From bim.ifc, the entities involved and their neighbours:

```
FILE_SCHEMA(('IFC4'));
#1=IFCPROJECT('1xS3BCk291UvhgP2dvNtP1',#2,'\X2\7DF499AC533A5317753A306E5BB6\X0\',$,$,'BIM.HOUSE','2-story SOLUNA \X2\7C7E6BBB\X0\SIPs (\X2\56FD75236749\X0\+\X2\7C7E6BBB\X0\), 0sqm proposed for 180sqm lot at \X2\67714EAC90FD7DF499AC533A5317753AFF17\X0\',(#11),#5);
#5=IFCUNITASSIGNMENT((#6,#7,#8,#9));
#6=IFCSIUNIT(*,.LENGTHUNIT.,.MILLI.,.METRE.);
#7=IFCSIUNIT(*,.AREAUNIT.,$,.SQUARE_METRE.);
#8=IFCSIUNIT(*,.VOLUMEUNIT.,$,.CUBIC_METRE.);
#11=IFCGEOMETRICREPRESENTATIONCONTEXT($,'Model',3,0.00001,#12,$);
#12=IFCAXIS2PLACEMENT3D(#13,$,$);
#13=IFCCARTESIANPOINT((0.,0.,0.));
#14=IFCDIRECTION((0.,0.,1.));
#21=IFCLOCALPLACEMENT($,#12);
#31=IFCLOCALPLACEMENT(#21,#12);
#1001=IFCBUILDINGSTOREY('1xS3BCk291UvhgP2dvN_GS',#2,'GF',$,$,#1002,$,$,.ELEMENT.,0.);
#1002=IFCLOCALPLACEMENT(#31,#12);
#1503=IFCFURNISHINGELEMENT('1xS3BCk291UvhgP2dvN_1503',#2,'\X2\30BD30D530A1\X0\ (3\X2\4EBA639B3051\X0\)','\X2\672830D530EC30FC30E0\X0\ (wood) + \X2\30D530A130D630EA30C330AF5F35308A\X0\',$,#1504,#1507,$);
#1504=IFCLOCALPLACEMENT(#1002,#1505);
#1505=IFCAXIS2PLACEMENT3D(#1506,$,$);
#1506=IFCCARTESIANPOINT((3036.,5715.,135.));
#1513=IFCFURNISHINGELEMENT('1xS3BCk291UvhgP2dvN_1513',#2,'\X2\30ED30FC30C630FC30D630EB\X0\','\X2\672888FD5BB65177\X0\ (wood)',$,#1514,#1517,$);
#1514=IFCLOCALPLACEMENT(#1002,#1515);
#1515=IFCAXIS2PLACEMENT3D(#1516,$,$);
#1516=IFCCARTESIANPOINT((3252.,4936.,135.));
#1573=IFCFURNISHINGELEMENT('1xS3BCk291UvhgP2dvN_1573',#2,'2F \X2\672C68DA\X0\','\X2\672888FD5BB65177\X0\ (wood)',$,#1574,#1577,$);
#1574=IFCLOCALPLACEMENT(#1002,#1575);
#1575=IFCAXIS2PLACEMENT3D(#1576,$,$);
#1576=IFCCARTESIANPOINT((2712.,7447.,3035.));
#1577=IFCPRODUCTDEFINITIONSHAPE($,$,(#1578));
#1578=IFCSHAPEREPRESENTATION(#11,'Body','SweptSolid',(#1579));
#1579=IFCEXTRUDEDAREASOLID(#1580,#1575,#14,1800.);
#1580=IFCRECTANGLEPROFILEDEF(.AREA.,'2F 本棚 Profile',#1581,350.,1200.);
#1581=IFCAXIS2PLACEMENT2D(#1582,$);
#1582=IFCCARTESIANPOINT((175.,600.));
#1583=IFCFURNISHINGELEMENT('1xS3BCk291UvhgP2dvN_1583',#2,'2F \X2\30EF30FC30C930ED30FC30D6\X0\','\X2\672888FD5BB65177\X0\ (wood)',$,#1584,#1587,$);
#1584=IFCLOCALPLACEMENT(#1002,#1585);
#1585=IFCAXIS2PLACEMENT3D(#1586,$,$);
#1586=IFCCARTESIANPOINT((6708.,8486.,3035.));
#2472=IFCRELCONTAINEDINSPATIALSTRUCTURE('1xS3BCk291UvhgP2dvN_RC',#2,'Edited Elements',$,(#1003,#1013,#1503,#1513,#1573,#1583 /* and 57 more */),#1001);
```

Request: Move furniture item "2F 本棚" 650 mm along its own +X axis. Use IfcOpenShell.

```python
import ifcopenshell
import ifcopenshell.api.geometry
import ifcopenshell.util.placement

model = ifcopenshell.open("bim.ifc")

item = model.by_id(1573)
matrix = ifcopenshell.util.placement.get_local_placement(item.ObjectPlacement)
matrix[:3, 3] += matrix[:3, 0] * 650.0
ifcopenshell.api.geometry.edit_object_placement(model, product=item, matrix=matrix, is_si=False)

print(ifcopenshell.util.placement.get_local_placement(item.ObjectPlacement).round(3) + 0.0)

model.write("bim_rev.ifc")
```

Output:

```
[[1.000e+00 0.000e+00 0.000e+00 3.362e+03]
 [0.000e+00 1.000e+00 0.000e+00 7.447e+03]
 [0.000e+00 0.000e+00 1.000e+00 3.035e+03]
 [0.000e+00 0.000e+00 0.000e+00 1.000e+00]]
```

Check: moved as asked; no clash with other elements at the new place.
